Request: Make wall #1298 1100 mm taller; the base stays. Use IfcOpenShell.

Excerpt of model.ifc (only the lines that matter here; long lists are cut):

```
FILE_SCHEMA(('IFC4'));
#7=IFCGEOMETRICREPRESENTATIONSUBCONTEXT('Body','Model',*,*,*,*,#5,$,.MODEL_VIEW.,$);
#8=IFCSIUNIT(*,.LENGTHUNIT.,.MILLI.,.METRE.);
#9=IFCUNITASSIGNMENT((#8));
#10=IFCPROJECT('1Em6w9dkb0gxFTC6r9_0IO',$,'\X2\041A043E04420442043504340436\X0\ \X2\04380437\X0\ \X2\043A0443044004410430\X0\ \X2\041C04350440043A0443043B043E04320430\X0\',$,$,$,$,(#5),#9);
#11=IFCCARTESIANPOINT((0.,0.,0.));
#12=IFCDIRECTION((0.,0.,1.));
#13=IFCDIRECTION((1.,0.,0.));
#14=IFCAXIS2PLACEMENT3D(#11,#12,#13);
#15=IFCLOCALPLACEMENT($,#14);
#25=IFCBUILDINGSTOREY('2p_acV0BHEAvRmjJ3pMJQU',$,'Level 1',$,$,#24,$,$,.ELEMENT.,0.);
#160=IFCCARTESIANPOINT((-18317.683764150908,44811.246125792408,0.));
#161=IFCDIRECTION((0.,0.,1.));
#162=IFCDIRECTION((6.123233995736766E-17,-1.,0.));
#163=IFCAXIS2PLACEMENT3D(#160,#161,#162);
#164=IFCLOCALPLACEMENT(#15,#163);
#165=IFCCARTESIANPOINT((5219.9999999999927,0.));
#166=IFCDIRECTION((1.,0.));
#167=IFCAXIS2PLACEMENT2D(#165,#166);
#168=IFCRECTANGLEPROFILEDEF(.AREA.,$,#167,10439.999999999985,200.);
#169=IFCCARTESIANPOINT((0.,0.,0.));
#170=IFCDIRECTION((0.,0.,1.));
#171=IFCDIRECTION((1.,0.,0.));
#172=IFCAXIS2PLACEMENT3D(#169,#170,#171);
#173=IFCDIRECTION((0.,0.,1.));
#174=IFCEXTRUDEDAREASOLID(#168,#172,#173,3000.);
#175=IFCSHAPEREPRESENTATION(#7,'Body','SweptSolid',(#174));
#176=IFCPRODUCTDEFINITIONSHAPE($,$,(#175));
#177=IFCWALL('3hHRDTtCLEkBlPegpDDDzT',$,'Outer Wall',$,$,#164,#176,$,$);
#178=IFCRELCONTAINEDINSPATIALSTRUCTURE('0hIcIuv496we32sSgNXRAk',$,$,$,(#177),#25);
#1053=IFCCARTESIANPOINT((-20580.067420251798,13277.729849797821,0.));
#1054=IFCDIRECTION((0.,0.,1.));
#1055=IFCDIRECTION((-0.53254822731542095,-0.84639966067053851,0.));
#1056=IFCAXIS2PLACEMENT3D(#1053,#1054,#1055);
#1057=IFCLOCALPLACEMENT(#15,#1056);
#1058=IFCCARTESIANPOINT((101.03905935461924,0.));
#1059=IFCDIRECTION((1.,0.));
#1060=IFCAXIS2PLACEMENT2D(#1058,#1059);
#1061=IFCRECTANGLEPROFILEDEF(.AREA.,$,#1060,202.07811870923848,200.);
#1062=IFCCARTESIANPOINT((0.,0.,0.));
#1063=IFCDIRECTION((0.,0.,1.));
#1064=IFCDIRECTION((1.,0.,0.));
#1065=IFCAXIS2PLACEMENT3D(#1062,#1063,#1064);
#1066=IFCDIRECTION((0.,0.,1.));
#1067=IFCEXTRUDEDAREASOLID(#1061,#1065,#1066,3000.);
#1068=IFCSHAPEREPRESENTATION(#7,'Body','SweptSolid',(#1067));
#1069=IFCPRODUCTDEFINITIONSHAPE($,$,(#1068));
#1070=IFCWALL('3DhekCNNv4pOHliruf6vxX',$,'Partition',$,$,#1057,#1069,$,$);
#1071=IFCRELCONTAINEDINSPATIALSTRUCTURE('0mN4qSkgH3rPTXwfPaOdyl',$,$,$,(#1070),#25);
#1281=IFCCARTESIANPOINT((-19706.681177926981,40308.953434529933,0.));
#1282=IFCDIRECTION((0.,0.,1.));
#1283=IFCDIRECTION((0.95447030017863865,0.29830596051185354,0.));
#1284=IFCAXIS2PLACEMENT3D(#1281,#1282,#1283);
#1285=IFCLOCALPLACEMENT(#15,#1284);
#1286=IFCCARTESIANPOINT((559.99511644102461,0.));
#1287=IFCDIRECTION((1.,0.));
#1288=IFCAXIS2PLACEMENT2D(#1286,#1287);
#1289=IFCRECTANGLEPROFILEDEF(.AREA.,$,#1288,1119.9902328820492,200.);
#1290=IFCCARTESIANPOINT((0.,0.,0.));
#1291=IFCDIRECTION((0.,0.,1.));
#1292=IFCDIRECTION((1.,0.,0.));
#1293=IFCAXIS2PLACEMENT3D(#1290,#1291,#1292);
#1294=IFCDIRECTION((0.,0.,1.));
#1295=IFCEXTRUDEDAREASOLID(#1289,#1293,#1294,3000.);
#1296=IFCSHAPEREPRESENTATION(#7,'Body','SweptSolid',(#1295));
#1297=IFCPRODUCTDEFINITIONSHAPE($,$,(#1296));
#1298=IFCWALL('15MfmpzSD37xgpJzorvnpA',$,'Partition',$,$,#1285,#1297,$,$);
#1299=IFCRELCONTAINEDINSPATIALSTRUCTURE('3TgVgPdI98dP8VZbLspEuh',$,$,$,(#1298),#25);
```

```python
import ifcopenshell
import ifcopenshell.geom
import ifcopenshell.util.representation
import ifcopenshell.util.shape
import ifcopenshell.util.unit

model = ifcopenshell.open("model.ifc")
unit_scale = ifcopenshell.util.unit.calculate_unit_scale(model)
settings = ifcopenshell.geom.settings()


def volume(element):
    """Net volume in cubic metres, openings subtracted."""
    shape = ifcopenshell.geom.create_shape(settings, element)
    return ifcopenshell.util.shape.get_volume(shape.geometry)


wall = model.by_id(1298)
before = volume(wall)

body = ifcopenshell.util.representation.get_representation(wall, "Model", "Body")
solid = body.Items[0]
old_height = solid.Depth
solid.Depth += 1.1 / unit_scale
after = volume(wall)

print(f"height {old_height:g} -> {solid.Depth:g}, volume {before:.3f} -> {after:.3f} m3")

model.write("model-out.ifc")
```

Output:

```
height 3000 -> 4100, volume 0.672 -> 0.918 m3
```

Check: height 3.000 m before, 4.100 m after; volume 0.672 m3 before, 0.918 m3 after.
